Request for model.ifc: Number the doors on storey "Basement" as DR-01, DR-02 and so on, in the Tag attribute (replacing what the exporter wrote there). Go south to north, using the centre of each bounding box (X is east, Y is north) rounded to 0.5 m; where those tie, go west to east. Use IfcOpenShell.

First a look at what the model holds.

```python
import ifcopenshell
import ifcopenshell.util.element
import ifcopenshell.util.placement

model = ifcopenshell.open("model.ifc")
print(model.schema)
storey = next(s for s in model.by_type("IfcBuildingStorey") if s.Name == "Basement")
doors = [e for e in ifcopenshell.util.element.get_decomposition(storey) if e.is_a("IfcDoor")]
for e in sorted(doors, key=lambda e: e.id()):
    origin = ifcopenshell.util.placement.get_local_placement(e.ObjectPlacement)[:3, 3]
    print(e.id(), e.Tag, e.Name, origin.round(2) + 0.0, sep=" | ")
```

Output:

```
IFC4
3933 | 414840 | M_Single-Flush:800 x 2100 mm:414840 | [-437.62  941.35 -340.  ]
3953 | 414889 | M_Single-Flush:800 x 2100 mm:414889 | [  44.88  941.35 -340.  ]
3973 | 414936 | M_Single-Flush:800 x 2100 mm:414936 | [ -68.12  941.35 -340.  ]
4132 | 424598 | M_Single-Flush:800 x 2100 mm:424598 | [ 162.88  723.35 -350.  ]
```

```python
import ifcopenshell
import ifcopenshell.geom
import ifcopenshell.util.element
import ifcopenshell.util.shape

model = ifcopenshell.open("model.ifc")
settings = ifcopenshell.geom.settings()
settings.set("use-world-coords", True)


def centre(element):
    shape = ifcopenshell.geom.create_shape(settings, element)
    return ifcopenshell.util.shape.get_bbox_centroid(shape.geometry)


storey = next(s for s in model.by_type("IfcBuildingStorey") if s.Name == "Basement")
doors = [e for e in ifcopenshell.util.element.get_decomposition(storey) if e.is_a("IfcDoor")]

# Insertion points can sit at a corner or the storey origin, so sort by the geometry (in metres).
centres = {e: centre(e) for e in doors}
doors.sort(key=lambda e: (round(centres[e][1] / 0.5), centres[e][0]))

for i, e in enumerate(doors, start=1):
    number = f"DR-{i:02d}"
    e.Tag = number
    print(e.id(), number)

model.write("model-out.ifc")
```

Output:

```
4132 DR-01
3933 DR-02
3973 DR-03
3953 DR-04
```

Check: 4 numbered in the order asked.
